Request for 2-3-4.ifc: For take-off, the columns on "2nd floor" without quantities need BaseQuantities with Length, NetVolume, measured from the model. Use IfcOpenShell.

First a look at what the model holds.

```python
import ifcopenshell
import ifcopenshell.util.element
import ifcopenshell.util.unit

model = ifcopenshell.open("2-3-4.ifc")
print(model.schema)
for unit_type in ("LENGTHUNIT", "AREAUNIT", "VOLUMEUNIT"):
    print(unit_type, ifcopenshell.util.unit.calculate_unit_scale(model, unit_type))
storey = next(s for s in model.by_type("IfcBuildingStorey") if s.Name == "2nd floor")
columns = [e for e in ifcopenshell.util.element.get_decomposition(storey) if e.is_a("IfcColumn")]
for e in sorted(columns, key=lambda e: e.id()):
    print(e.id(), e.is_a(), e.Name, list(ifcopenshell.util.element.get_psets(e, qtos_only=True)), sep=" | ")
```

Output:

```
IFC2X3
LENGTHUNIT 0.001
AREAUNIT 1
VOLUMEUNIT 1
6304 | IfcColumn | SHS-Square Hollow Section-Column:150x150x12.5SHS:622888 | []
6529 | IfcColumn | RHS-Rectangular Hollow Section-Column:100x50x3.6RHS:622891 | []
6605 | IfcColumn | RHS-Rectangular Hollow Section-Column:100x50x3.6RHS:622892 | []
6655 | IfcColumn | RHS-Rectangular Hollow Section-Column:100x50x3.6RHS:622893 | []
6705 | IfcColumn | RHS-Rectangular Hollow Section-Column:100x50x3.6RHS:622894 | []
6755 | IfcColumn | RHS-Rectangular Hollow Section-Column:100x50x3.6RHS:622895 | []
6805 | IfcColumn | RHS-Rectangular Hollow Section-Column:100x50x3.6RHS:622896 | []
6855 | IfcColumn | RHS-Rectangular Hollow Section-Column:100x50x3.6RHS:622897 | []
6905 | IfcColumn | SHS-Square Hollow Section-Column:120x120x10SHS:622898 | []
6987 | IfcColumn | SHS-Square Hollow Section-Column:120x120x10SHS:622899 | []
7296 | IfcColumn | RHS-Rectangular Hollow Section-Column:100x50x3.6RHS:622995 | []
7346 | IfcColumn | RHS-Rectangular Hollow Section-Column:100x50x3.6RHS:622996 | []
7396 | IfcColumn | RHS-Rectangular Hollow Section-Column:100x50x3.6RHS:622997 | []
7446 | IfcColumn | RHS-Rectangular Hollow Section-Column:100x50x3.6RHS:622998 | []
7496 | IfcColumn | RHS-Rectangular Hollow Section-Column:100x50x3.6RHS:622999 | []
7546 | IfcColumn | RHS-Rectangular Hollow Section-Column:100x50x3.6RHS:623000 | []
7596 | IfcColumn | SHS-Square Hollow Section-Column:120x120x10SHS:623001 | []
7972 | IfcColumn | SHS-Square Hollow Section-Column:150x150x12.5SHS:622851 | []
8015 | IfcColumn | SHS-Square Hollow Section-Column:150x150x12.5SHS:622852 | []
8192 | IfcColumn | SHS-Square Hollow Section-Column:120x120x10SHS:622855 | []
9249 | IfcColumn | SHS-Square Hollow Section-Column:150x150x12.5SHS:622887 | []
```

```python
import ifcopenshell
import ifcopenshell.api.pset
import ifcopenshell.geom
import ifcopenshell.util.element
import ifcopenshell.util.shape
import ifcopenshell.util.unit

model = ifcopenshell.open("2-3-4.ifc")
unit_scale = ifcopenshell.util.unit.calculate_unit_scale(model)
volume_scale = ifcopenshell.util.unit.calculate_unit_scale(model, "VOLUMEUNIT")
settings = ifcopenshell.geom.settings()

storey = next(s for s in model.by_type("IfcBuildingStorey") if s.Name == "2nd floor")
columns = [e for e in ifcopenshell.util.element.get_decomposition(storey) if e.is_a("IfcColumn")]

for e in sorted(columns, key=lambda e: e.id()):
    if ifcopenshell.util.element.get_psets(e, qtos_only=True, should_inherit=False):
        continue
    # Geometry comes back in metres, in the element's own axes.
    shape = ifcopenshell.geom.create_shape(settings, e)
    values = {
        "Length": ifcopenshell.util.shape.get_z(shape.geometry) / unit_scale,
        "NetVolume": ifcopenshell.util.shape.get_volume(shape.geometry) / volume_scale,
    }
    qto = ifcopenshell.api.pset.add_qto(model, product=e, name="BaseQuantities")
    ifcopenshell.api.pset.edit_qto(model, qto=qto, properties=values)
    print(e.id(), {k: round(v, 3) for k, v in values.items()})

model.write("2-3-4_updated.ifc")
```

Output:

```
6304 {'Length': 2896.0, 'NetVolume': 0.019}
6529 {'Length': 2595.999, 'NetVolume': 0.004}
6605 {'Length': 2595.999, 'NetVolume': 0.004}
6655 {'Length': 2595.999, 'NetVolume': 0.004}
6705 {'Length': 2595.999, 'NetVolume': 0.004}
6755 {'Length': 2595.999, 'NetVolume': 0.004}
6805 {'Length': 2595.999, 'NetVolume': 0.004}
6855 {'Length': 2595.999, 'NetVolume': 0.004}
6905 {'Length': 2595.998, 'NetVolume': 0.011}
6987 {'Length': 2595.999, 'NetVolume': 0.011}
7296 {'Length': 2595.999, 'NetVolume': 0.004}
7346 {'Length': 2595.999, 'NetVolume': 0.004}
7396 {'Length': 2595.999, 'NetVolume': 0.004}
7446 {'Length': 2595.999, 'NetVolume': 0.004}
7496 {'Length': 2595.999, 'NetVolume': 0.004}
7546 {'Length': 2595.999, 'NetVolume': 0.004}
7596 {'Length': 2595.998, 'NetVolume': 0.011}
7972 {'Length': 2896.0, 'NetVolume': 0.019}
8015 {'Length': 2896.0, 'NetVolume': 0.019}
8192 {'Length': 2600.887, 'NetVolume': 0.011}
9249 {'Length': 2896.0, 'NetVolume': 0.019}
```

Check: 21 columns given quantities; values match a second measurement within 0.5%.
